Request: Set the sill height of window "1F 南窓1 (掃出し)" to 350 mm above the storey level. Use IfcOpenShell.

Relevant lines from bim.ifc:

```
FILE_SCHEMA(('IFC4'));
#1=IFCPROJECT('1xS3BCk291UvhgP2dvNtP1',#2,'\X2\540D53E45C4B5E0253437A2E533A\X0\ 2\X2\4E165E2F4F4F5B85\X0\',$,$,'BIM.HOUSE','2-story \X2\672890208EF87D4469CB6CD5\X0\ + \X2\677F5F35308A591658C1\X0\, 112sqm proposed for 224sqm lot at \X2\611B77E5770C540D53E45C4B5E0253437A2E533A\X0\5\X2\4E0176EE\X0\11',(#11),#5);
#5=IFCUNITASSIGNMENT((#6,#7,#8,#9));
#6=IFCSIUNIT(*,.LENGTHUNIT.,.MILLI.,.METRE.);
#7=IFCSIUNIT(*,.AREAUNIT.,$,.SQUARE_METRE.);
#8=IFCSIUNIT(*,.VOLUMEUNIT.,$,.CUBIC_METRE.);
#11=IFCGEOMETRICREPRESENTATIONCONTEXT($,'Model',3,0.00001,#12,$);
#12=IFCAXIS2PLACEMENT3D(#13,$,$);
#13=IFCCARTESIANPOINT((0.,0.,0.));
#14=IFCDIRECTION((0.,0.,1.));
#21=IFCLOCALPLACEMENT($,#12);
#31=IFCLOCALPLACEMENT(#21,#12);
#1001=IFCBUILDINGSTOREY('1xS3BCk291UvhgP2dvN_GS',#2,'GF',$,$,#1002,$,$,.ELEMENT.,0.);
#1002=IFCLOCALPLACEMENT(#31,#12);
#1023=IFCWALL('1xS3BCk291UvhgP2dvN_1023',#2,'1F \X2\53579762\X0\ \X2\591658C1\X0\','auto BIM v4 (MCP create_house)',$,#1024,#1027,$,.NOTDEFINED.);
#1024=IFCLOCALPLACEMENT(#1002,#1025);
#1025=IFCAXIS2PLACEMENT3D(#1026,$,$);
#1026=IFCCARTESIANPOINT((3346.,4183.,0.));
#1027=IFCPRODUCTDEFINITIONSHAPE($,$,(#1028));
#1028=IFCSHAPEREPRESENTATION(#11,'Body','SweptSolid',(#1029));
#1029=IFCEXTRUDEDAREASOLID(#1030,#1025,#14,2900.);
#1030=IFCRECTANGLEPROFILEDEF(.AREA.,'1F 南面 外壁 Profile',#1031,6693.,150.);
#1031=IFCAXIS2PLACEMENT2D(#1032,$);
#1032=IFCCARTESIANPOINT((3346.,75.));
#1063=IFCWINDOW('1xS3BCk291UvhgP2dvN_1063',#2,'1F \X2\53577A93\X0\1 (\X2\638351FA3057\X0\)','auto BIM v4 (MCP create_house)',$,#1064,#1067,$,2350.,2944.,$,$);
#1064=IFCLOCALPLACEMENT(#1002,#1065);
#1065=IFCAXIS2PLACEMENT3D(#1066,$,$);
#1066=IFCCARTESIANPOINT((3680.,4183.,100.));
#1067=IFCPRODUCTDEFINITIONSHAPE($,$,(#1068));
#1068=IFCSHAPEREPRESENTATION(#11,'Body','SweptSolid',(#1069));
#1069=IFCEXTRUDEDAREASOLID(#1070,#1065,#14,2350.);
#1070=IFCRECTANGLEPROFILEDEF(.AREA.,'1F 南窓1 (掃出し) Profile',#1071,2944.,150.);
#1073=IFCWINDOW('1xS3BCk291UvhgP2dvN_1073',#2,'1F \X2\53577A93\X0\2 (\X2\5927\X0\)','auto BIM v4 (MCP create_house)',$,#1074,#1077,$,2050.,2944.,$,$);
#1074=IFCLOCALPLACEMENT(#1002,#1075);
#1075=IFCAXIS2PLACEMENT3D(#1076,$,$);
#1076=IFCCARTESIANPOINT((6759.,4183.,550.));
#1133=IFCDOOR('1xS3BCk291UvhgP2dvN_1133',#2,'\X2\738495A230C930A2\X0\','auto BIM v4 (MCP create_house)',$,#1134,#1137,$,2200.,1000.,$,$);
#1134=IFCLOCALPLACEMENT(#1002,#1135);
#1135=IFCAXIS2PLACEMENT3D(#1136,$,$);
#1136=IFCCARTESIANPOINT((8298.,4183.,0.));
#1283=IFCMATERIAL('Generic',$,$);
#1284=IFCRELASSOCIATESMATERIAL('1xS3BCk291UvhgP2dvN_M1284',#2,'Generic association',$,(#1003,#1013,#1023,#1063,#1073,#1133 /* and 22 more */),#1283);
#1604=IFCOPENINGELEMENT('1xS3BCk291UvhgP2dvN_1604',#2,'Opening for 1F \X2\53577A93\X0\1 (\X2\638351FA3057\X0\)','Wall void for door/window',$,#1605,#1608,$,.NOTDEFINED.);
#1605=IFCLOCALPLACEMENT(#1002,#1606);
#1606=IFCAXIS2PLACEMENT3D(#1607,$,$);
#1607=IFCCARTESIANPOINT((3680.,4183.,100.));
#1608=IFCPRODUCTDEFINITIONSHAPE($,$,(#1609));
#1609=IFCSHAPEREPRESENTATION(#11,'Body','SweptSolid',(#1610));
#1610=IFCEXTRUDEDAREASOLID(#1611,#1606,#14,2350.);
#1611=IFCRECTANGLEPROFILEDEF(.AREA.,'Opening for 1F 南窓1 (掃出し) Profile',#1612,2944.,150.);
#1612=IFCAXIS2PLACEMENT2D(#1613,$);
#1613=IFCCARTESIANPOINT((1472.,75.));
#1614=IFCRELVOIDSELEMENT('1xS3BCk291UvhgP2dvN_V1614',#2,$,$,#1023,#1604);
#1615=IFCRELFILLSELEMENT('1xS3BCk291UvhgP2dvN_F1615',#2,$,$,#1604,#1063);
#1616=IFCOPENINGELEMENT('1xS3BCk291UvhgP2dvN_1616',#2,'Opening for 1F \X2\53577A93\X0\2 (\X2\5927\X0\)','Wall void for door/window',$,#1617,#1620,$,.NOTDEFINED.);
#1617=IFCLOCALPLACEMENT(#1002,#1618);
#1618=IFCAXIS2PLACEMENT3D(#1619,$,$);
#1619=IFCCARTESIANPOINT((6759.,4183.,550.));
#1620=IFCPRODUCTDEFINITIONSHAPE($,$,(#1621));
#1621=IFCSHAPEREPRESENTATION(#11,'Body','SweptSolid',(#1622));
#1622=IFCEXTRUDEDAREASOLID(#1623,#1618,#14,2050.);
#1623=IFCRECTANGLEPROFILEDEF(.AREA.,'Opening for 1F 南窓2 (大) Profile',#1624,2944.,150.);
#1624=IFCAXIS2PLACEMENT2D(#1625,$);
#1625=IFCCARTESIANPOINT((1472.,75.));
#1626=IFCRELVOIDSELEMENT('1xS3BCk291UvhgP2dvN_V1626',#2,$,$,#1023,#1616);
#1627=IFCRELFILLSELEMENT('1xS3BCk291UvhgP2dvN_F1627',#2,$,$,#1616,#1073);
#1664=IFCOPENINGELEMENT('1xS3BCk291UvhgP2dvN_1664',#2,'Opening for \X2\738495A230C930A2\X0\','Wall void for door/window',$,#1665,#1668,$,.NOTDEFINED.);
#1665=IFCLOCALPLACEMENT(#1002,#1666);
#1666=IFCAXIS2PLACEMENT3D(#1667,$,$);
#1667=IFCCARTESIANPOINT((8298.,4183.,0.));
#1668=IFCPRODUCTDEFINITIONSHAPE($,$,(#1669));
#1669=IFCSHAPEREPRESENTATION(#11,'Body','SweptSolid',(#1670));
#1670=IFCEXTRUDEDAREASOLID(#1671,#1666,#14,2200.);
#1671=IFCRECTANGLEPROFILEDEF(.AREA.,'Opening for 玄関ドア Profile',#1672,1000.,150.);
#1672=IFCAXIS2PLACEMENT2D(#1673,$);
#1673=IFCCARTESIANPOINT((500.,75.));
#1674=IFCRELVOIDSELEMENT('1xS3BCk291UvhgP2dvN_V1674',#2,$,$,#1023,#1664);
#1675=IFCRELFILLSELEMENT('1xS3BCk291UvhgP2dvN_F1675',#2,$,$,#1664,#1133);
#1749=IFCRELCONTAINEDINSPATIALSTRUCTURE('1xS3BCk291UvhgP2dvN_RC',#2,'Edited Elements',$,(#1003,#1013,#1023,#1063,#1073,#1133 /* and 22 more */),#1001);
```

```python
import numpy as np
import ifcopenshell
import ifcopenshell.api.geometry
import ifcopenshell.geom
import ifcopenshell.util.element
import ifcopenshell.util.placement
import ifcopenshell.util.shape
import ifcopenshell.util.unit

model = ifcopenshell.open("bim.ifc")
unit_scale = ifcopenshell.util.unit.calculate_unit_scale(model)

window = model.by_guid("1xS3BCk291UvhgP2dvN_1063")
opening = window.FillsVoids[0].RelatingOpeningElement
storey = ifcopenshell.util.element.get_container(window, ifc_class="IfcBuildingStorey")
level = ifcopenshell.util.placement.get_local_placement(storey.ObjectPlacement)[2, 3]

# The opening's origin need not be at the sill, so measure its lowest point.
shape = ifcopenshell.geom.create_shape(ifcopenshell.geom.settings(), opening)
bottom = ifcopenshell.util.shape.get_shape_bottom_elevation(shape, shape.geometry) / unit_scale
dz = level + 0.35 / unit_scale - bottom

shift = np.array([0.0, 0.0, dz])
# The window is not placed relative to its opening, so move both.
for product in (opening, window):
    matrix = ifcopenshell.util.placement.get_local_placement(product.ObjectPlacement)
    matrix[:3, 3] += shift
    ifcopenshell.api.geometry.edit_object_placement(model, product=product, matrix=matrix, is_si=False)

print(f"moved by {dz * unit_scale:+.3f} m")

model.write("bim_edited.ifc")
```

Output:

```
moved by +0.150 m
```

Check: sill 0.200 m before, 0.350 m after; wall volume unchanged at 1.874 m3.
